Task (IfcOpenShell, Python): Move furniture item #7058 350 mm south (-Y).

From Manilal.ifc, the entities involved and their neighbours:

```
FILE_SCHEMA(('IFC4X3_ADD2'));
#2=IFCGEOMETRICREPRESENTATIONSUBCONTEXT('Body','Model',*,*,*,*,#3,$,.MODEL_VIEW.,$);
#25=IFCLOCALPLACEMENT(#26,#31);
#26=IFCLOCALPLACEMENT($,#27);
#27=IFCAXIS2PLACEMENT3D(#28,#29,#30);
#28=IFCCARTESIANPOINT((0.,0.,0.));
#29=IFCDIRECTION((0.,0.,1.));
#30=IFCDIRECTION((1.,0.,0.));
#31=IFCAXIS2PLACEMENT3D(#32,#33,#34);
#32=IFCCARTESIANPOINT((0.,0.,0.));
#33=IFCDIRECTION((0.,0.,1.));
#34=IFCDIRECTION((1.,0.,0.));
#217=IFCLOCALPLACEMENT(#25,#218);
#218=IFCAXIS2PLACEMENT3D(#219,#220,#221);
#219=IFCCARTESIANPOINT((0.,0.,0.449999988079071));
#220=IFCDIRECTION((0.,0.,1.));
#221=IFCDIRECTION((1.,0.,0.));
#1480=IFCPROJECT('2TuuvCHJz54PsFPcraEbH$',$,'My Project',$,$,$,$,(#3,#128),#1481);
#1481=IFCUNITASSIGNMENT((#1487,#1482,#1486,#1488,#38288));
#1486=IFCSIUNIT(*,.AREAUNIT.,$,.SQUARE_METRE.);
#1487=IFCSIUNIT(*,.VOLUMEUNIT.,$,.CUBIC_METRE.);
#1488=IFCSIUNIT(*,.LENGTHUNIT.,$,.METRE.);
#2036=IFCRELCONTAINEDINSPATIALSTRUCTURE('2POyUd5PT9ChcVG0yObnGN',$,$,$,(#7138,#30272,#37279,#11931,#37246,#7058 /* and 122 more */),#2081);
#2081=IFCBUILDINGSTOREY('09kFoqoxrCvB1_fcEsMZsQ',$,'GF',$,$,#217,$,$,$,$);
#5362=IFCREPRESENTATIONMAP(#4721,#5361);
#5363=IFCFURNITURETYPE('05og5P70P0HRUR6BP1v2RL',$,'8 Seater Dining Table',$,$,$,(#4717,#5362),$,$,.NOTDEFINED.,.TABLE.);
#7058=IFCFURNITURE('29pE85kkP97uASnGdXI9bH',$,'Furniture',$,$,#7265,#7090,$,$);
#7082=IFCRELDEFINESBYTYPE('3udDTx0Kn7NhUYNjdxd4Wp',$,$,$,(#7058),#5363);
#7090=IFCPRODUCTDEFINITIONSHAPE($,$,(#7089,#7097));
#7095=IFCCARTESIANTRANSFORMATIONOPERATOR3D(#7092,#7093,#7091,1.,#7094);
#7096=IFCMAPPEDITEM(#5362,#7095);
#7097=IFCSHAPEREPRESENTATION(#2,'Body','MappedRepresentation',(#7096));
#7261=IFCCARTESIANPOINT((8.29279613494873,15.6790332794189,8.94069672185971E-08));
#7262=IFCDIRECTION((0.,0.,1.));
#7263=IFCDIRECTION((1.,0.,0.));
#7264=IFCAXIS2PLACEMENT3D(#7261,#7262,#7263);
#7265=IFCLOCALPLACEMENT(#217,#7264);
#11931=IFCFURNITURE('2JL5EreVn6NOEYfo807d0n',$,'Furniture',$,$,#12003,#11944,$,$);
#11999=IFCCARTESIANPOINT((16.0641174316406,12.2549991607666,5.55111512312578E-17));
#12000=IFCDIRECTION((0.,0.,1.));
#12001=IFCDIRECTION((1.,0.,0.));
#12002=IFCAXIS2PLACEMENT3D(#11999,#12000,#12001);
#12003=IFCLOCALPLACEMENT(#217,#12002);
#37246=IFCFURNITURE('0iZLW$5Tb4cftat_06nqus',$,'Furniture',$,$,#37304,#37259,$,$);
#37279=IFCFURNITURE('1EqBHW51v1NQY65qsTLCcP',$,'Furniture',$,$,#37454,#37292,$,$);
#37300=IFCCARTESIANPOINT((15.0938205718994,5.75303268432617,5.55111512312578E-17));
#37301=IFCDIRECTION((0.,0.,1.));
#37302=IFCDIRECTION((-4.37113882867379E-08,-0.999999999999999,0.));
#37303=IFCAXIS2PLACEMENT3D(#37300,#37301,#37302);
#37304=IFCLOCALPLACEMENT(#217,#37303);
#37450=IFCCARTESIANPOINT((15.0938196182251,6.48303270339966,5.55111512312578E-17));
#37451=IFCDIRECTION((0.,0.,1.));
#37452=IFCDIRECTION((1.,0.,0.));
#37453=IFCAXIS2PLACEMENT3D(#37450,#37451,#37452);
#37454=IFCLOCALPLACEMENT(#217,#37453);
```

```python
import ifcopenshell
import ifcopenshell.api.geometry
import ifcopenshell.util.placement
import ifcopenshell.util.unit

model = ifcopenshell.open("Manilal.ifc")
unit_scale = ifcopenshell.util.unit.calculate_unit_scale(model)

item = model.by_guid("29pE85kkP97uASnGdXI9bH")
matrix = ifcopenshell.util.placement.get_local_placement(item.ObjectPlacement)
matrix[1, 3] -= 0.35 / unit_scale
ifcopenshell.api.geometry.edit_object_placement(model, product=item, matrix=matrix, is_si=False)

print(ifcopenshell.util.placement.get_local_placement(item.ObjectPlacement).round(3) + 0.0)

model.write("Manilal_updated.ifc")
```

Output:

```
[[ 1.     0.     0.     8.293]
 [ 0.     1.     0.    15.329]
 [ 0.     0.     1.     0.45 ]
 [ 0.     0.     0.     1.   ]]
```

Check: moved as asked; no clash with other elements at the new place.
